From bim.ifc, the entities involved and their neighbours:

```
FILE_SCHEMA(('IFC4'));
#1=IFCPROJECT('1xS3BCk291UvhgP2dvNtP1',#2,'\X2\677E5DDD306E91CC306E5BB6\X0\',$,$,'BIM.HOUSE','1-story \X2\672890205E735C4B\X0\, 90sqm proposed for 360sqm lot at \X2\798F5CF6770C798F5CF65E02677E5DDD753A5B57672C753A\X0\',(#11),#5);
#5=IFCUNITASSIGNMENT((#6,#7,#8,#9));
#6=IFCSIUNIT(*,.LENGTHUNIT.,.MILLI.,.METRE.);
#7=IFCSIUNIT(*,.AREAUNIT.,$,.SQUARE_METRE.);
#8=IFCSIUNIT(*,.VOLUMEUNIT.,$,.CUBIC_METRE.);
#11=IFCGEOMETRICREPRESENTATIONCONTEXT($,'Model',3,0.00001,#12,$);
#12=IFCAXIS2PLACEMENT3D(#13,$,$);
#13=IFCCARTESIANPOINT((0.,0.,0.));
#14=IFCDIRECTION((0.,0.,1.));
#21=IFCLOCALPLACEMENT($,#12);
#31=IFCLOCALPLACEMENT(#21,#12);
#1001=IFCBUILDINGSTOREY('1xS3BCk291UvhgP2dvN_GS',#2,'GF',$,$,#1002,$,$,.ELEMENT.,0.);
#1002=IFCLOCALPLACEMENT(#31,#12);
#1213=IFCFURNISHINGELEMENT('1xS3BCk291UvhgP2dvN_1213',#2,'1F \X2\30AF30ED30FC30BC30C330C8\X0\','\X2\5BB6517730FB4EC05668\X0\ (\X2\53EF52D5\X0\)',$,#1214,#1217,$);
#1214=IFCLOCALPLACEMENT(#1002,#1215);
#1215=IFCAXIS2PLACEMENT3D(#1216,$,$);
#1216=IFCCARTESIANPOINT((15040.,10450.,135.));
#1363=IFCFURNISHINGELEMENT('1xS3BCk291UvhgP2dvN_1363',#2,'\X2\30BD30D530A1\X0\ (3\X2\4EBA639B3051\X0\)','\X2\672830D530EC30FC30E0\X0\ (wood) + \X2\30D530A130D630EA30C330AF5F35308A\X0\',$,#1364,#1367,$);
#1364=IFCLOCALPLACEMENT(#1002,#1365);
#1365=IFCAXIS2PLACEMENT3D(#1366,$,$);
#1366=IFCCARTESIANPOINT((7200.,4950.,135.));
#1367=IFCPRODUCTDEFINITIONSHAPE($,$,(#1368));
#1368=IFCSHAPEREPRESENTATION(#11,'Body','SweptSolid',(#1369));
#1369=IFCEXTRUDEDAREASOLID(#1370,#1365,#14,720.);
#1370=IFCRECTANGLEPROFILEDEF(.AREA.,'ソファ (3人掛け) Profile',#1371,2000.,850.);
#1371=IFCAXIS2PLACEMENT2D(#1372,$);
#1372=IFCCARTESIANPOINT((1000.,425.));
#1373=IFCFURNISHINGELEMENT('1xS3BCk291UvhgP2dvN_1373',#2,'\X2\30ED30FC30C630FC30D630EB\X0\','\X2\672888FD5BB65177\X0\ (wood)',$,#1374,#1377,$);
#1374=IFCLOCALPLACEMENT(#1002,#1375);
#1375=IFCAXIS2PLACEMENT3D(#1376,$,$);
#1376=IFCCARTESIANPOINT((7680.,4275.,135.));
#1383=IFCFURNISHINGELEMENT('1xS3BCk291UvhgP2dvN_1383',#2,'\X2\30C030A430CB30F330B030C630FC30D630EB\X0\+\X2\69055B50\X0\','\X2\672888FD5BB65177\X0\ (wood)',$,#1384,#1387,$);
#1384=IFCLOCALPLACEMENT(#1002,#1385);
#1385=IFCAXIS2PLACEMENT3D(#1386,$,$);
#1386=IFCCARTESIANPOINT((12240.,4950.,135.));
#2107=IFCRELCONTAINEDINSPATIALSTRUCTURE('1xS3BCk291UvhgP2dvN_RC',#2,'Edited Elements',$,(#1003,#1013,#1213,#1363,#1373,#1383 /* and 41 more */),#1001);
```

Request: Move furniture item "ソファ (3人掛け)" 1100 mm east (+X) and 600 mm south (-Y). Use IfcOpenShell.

```python
import ifcopenshell
import ifcopenshell.api.geometry
import ifcopenshell.util.placement
import ifcopenshell.util.unit

model = ifcopenshell.open("bim.ifc")
unit_scale = ifcopenshell.util.unit.calculate_unit_scale(model)

item = model.by_id(1363)
matrix = ifcopenshell.util.placement.get_local_placement(item.ObjectPlacement)
matrix[0, 3] += 1.1 / unit_scale
matrix[1, 3] -= 0.6 / unit_scale
ifcopenshell.api.geometry.edit_object_placement(model, product=item, matrix=matrix, is_si=False)

print(ifcopenshell.util.placement.get_local_placement(item.ObjectPlacement).round(3) + 0.0)

model.write("bim_edited.ifc")
```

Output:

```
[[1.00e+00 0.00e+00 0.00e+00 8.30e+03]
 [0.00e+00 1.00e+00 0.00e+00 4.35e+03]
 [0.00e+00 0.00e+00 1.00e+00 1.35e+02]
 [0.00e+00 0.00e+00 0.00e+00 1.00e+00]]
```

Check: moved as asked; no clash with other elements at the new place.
